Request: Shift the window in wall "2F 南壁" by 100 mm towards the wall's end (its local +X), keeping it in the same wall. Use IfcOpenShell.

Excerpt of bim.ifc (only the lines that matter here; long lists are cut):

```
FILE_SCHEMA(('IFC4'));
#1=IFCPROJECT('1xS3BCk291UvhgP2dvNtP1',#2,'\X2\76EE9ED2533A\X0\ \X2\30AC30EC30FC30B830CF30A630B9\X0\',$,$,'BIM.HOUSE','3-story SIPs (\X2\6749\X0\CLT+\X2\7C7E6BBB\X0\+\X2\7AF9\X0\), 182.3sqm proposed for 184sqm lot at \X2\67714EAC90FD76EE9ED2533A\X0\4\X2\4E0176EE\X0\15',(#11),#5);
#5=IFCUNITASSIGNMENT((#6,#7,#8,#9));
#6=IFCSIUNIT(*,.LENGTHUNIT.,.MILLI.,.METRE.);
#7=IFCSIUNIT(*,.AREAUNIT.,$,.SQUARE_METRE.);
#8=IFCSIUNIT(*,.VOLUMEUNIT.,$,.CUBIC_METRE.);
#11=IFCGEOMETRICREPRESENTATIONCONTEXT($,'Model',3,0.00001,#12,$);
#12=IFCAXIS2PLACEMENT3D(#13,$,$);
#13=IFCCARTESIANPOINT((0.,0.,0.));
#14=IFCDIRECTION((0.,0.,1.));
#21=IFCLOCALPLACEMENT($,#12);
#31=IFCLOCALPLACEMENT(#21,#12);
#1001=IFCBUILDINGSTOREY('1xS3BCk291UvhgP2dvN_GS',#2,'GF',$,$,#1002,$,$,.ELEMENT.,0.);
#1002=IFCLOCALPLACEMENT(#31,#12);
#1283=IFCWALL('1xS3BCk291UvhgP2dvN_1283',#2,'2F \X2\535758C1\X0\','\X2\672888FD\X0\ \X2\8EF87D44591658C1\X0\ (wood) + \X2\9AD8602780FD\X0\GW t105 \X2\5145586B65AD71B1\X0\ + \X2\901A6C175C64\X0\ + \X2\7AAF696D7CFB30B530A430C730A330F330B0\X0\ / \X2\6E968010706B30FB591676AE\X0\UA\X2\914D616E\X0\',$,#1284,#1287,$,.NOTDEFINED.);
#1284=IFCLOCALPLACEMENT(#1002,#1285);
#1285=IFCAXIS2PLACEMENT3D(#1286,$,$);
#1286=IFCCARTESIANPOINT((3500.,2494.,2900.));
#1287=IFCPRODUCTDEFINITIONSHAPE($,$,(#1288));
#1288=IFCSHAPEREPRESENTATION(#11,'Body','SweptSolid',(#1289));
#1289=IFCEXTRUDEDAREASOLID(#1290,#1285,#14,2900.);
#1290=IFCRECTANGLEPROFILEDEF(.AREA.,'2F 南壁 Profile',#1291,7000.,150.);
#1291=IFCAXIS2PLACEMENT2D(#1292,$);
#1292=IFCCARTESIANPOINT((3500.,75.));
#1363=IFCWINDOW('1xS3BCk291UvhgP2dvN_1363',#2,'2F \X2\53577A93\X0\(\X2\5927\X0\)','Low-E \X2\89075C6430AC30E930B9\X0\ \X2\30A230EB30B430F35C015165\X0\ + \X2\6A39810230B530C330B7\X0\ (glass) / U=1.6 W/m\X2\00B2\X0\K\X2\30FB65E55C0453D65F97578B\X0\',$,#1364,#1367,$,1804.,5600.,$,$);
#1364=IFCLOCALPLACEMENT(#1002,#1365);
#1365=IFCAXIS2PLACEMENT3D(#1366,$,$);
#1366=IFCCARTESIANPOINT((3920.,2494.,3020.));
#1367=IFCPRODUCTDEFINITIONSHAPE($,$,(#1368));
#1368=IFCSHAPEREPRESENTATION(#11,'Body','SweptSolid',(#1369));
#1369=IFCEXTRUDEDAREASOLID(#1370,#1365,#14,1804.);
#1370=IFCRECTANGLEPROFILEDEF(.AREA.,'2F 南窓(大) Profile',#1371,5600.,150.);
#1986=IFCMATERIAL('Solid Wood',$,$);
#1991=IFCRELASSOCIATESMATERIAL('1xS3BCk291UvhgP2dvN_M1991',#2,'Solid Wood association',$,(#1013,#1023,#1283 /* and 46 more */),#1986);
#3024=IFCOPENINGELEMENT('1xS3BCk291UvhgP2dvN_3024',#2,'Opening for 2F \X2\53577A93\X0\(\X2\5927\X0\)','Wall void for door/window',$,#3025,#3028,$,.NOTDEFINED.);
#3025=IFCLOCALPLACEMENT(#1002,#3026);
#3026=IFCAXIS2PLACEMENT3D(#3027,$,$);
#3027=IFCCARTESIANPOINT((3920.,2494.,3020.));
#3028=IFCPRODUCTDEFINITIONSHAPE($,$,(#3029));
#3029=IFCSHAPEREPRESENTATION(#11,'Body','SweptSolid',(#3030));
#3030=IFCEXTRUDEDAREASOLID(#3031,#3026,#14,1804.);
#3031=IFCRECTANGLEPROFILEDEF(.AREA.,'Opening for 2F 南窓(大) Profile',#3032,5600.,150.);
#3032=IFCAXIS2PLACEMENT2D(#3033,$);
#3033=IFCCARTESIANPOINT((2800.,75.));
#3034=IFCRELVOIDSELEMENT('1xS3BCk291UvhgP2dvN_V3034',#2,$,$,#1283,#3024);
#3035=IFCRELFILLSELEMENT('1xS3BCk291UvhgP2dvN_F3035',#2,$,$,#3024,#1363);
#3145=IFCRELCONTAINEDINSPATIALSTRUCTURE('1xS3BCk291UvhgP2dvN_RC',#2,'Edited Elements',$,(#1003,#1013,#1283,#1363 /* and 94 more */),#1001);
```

```python
import ifcopenshell
import ifcopenshell.api.geometry
import ifcopenshell.util.placement
import ifcopenshell.util.unit

model = ifcopenshell.open("bim.ifc")
unit_scale = ifcopenshell.util.unit.calculate_unit_scale(model)

window = model.by_guid("1xS3BCk291UvhgP2dvN_1363")
opening = window.FillsVoids[0].RelatingOpeningElement
wall = opening.VoidsElements[0].RelatingBuildingElement

wall_matrix = ifcopenshell.util.placement.get_local_placement(wall.ObjectPlacement)
shift = wall_matrix[:3, 0] * 0.1 / unit_scale
before = ifcopenshell.util.placement.get_local_placement(window.ObjectPlacement)[:3, 3].copy()

# The window is not placed relative to its opening, so move both.
for product in (opening, window):
    matrix = ifcopenshell.util.placement.get_local_placement(product.ObjectPlacement)
    matrix[:3, 3] += shift
    ifcopenshell.api.geometry.edit_object_placement(model, product=product, matrix=matrix, is_si=False)

after = ifcopenshell.util.placement.get_local_placement(window.ObjectPlacement)[:3, 3]
print("window moved by", (after - before).round(3) + 0.0)

model.write("bim_rev.ifc")
```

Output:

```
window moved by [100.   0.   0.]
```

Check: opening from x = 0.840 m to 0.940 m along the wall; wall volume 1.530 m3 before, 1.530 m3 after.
